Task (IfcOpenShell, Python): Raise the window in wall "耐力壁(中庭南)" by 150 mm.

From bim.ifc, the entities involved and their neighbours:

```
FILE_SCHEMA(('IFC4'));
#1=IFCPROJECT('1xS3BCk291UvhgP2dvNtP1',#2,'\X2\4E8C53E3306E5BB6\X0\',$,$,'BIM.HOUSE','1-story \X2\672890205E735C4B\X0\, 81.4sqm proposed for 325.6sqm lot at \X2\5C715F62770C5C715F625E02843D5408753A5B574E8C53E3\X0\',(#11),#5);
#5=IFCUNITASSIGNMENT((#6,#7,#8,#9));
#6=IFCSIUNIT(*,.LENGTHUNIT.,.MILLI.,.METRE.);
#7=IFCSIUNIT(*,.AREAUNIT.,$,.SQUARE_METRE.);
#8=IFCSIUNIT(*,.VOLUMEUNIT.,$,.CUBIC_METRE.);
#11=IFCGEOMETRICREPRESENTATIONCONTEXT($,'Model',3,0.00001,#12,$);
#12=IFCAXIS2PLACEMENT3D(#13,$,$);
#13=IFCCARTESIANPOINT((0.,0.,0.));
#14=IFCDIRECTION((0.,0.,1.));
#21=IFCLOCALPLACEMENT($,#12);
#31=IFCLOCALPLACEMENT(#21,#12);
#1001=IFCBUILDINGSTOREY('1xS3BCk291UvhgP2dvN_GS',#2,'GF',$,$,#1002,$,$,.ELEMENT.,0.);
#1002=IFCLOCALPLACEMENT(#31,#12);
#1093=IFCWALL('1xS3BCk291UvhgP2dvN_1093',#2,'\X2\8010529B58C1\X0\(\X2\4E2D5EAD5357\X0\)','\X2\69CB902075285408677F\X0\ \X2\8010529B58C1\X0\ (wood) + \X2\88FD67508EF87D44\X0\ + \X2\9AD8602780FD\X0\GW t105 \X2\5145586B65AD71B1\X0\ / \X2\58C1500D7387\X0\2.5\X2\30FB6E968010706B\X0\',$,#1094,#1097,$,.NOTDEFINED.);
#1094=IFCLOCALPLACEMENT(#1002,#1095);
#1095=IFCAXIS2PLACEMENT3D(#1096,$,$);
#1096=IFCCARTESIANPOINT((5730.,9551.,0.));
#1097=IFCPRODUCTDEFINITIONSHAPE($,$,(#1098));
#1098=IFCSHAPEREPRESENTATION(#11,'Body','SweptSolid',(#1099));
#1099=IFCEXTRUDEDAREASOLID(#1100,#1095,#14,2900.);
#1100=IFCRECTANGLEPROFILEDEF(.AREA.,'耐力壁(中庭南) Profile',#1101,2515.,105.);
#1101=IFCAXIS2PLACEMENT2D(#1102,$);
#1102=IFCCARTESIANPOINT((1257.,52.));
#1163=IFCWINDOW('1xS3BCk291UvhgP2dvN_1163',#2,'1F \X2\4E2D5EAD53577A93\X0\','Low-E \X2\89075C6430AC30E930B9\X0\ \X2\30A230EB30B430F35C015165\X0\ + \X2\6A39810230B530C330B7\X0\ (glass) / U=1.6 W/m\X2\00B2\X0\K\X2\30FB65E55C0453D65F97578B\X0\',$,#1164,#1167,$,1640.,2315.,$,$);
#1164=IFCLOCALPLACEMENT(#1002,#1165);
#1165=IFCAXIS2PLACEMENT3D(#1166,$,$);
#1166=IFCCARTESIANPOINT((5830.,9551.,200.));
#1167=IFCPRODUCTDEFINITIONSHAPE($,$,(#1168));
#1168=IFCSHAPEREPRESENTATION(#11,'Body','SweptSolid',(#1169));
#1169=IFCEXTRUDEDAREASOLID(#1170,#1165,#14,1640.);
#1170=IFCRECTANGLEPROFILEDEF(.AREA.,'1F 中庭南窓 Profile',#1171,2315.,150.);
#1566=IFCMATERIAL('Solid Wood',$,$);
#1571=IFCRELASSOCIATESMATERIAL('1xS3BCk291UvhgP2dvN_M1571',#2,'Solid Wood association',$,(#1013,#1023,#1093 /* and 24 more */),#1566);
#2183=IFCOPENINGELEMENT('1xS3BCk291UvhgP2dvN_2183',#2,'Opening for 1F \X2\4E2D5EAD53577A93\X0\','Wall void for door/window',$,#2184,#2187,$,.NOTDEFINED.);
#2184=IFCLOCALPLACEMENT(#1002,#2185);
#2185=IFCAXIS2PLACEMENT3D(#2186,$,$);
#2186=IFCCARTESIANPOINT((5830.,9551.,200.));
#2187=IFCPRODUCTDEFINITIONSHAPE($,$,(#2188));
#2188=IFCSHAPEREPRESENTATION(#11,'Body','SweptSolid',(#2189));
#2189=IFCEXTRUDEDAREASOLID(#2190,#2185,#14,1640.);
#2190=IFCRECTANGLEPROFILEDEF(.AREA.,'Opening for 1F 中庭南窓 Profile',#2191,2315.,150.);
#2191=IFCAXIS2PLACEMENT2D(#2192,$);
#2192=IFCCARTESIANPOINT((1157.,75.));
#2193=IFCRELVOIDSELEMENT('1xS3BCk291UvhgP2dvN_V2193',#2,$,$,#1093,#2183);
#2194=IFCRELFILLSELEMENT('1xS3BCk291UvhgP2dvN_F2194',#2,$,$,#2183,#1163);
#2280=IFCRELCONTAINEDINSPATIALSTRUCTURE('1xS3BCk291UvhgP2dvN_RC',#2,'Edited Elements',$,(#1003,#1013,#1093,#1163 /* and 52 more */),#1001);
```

```python
import numpy as np
import ifcopenshell
import ifcopenshell.api.geometry
import ifcopenshell.util.placement
import ifcopenshell.util.unit

model = ifcopenshell.open("bim.ifc")
unit_scale = ifcopenshell.util.unit.calculate_unit_scale(model)

window = model.by_guid("1xS3BCk291UvhgP2dvN_1163")
opening = window.FillsVoids[0].RelatingOpeningElement
dz = 150.0

shift = np.array([0.0, 0.0, dz])
# The window is not placed relative to its opening, so move both.
for product in (opening, window):
    matrix = ifcopenshell.util.placement.get_local_placement(product.ObjectPlacement)
    matrix[:3, 3] += shift
    ifcopenshell.api.geometry.edit_object_placement(model, product=product, matrix=matrix, is_si=False)

print(f"moved by {dz * unit_scale:+.3f} m")

model.write("bim_v2.ifc")
```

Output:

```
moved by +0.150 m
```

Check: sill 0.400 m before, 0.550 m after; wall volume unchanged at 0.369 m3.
